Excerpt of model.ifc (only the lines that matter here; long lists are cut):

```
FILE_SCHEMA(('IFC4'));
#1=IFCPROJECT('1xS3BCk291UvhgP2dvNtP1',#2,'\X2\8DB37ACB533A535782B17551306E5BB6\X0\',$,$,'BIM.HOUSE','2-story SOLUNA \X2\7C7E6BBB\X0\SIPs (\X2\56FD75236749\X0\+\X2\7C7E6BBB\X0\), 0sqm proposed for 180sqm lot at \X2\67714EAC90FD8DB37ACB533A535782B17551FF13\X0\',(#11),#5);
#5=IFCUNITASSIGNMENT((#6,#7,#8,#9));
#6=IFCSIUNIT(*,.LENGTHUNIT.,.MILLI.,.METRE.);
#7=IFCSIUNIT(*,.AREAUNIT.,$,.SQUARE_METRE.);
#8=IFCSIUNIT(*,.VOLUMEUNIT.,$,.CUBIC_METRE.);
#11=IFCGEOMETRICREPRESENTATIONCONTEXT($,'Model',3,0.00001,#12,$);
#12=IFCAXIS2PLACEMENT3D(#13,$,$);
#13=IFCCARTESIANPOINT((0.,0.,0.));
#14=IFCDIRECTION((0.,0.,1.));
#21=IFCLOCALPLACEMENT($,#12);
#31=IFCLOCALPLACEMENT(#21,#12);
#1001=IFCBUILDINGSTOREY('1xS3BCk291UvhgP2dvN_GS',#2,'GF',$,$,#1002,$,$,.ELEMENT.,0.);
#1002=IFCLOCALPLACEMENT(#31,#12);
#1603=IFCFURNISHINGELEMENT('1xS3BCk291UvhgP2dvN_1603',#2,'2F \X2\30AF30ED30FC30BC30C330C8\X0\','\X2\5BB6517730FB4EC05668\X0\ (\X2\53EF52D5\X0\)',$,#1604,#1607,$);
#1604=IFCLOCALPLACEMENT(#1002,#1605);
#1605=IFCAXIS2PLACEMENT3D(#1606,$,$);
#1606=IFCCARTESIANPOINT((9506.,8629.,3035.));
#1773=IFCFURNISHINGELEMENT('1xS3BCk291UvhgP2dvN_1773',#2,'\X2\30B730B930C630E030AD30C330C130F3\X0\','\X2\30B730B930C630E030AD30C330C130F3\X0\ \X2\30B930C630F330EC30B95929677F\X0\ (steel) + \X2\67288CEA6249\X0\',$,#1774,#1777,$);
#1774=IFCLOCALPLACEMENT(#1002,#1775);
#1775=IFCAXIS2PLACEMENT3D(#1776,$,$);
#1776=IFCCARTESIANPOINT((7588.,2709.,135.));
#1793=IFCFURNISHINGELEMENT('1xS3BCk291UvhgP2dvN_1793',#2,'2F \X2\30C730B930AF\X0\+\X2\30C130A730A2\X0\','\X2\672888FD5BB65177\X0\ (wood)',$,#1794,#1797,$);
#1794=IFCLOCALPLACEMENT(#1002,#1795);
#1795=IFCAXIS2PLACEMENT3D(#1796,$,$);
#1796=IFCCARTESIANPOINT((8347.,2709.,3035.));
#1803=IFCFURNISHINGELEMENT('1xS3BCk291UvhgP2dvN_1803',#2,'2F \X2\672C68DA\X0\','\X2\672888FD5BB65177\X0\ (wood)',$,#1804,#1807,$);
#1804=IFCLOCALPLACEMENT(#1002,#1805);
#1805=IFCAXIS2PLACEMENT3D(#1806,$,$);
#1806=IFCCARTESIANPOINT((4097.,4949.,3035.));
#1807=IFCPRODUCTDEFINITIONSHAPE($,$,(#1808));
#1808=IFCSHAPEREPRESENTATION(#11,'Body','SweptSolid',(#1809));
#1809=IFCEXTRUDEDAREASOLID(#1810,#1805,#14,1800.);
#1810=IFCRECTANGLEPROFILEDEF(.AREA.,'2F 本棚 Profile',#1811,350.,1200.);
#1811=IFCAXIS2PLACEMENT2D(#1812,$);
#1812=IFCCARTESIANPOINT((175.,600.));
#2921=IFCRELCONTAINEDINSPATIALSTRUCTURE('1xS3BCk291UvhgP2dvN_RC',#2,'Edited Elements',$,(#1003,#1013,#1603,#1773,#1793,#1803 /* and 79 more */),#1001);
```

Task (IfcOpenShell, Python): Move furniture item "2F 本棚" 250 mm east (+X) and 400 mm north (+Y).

```python
import ifcopenshell
import ifcopenshell.api.geometry
import ifcopenshell.util.placement
import ifcopenshell.util.unit

model = ifcopenshell.open("model.ifc")
unit_scale = ifcopenshell.util.unit.calculate_unit_scale(model)

item = model.by_guid("1xS3BCk291UvhgP2dvN_1803")
matrix = ifcopenshell.util.placement.get_local_placement(item.ObjectPlacement)
matrix[0, 3] += 0.25 / unit_scale
matrix[1, 3] += 0.4 / unit_scale
ifcopenshell.api.geometry.edit_object_placement(model, product=item, matrix=matrix, is_si=False)

print(ifcopenshell.util.placement.get_local_placement(item.ObjectPlacement).round(3) + 0.0)

model.write("model_rev.ifc")
```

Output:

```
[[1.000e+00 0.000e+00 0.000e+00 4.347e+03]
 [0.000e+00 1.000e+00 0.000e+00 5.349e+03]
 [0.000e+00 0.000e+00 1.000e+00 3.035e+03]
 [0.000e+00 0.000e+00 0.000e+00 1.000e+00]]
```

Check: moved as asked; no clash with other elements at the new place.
